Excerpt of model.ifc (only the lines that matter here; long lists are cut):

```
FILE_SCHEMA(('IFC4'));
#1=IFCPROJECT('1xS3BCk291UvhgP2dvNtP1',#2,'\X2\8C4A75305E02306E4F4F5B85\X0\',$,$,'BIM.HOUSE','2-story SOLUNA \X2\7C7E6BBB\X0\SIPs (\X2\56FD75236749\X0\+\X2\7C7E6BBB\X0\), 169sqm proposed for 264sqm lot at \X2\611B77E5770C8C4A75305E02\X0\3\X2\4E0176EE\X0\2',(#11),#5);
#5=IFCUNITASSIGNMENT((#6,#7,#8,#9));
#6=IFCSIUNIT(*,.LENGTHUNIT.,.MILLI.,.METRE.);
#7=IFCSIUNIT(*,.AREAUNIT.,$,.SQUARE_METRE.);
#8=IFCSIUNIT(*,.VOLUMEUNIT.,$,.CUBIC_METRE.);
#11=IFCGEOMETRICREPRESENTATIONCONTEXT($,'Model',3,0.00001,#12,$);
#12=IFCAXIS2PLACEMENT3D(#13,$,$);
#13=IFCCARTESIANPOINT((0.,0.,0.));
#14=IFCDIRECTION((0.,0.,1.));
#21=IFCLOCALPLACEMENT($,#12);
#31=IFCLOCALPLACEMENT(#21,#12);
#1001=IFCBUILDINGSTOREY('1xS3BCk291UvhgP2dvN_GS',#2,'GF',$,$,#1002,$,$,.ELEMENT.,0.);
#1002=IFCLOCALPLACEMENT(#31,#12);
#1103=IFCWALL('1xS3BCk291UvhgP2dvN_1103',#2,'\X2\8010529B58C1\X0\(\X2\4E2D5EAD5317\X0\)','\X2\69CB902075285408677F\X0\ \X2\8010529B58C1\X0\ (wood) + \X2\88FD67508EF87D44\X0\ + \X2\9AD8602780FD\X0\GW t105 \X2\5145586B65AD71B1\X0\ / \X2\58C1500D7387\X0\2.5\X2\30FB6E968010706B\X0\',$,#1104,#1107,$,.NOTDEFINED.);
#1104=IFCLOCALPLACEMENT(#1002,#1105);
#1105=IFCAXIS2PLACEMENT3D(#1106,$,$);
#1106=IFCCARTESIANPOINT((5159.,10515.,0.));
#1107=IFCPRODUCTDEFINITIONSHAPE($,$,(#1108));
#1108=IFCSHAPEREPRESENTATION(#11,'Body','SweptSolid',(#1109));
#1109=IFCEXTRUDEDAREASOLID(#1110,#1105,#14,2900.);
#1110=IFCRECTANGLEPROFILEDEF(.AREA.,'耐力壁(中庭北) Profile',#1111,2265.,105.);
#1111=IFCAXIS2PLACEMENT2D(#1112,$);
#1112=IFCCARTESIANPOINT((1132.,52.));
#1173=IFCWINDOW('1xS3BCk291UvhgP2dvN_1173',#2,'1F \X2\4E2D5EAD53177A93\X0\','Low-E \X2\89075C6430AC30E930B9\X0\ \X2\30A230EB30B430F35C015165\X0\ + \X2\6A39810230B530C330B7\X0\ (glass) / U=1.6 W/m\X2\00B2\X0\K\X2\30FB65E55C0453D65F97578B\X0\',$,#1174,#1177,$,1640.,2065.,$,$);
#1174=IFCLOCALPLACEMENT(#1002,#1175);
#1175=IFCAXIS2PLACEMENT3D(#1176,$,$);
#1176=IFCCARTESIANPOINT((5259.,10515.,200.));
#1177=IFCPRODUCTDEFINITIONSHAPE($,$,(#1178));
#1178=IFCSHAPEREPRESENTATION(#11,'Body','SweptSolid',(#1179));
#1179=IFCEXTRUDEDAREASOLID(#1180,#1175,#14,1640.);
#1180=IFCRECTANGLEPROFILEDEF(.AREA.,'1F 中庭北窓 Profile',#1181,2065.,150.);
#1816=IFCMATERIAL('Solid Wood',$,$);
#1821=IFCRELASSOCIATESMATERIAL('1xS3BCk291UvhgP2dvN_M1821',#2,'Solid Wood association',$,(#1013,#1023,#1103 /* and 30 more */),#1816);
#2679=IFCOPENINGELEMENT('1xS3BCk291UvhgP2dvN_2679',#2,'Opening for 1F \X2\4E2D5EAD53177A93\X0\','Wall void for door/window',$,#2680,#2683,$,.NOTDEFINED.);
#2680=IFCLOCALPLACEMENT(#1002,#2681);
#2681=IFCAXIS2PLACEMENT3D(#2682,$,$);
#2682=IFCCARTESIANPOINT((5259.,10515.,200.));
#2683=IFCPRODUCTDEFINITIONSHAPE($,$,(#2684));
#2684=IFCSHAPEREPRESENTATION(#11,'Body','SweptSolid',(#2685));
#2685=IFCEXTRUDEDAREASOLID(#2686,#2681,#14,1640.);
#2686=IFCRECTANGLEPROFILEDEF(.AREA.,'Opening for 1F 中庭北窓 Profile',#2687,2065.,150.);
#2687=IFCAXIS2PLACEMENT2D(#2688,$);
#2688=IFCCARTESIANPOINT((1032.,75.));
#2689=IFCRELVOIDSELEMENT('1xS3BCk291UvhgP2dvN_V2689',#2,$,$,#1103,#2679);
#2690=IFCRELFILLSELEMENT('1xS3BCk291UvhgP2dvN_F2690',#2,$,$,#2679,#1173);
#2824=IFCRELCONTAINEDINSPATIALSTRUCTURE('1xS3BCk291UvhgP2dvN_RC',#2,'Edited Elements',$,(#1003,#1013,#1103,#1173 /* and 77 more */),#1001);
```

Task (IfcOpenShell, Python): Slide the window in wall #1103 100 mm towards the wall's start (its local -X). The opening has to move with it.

```python
import ifcopenshell
import ifcopenshell.api.geometry
import ifcopenshell.util.placement
import ifcopenshell.util.unit

model = ifcopenshell.open("model.ifc")
unit_scale = ifcopenshell.util.unit.calculate_unit_scale(model)

window = model.by_id(1173)
opening = window.FillsVoids[0].RelatingOpeningElement
wall = opening.VoidsElements[0].RelatingBuildingElement

wall_matrix = ifcopenshell.util.placement.get_local_placement(wall.ObjectPlacement)
shift = wall_matrix[:3, 0] * -0.1 / unit_scale
before = ifcopenshell.util.placement.get_local_placement(window.ObjectPlacement)[:3, 3].copy()

# The window is not placed relative to its opening, so move both.
for product in (opening, window):
    matrix = ifcopenshell.util.placement.get_local_placement(product.ObjectPlacement)
    matrix[:3, 3] += shift
    ifcopenshell.api.geometry.edit_object_placement(model, product=product, matrix=matrix, is_si=False)

after = ifcopenshell.util.placement.get_local_placement(window.ObjectPlacement)[:3, 3]
print("window moved by", (after - before).round(3) + 0.0)

model.write("model-out.ifc")
```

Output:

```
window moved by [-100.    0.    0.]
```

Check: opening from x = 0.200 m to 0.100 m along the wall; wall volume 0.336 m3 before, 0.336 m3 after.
